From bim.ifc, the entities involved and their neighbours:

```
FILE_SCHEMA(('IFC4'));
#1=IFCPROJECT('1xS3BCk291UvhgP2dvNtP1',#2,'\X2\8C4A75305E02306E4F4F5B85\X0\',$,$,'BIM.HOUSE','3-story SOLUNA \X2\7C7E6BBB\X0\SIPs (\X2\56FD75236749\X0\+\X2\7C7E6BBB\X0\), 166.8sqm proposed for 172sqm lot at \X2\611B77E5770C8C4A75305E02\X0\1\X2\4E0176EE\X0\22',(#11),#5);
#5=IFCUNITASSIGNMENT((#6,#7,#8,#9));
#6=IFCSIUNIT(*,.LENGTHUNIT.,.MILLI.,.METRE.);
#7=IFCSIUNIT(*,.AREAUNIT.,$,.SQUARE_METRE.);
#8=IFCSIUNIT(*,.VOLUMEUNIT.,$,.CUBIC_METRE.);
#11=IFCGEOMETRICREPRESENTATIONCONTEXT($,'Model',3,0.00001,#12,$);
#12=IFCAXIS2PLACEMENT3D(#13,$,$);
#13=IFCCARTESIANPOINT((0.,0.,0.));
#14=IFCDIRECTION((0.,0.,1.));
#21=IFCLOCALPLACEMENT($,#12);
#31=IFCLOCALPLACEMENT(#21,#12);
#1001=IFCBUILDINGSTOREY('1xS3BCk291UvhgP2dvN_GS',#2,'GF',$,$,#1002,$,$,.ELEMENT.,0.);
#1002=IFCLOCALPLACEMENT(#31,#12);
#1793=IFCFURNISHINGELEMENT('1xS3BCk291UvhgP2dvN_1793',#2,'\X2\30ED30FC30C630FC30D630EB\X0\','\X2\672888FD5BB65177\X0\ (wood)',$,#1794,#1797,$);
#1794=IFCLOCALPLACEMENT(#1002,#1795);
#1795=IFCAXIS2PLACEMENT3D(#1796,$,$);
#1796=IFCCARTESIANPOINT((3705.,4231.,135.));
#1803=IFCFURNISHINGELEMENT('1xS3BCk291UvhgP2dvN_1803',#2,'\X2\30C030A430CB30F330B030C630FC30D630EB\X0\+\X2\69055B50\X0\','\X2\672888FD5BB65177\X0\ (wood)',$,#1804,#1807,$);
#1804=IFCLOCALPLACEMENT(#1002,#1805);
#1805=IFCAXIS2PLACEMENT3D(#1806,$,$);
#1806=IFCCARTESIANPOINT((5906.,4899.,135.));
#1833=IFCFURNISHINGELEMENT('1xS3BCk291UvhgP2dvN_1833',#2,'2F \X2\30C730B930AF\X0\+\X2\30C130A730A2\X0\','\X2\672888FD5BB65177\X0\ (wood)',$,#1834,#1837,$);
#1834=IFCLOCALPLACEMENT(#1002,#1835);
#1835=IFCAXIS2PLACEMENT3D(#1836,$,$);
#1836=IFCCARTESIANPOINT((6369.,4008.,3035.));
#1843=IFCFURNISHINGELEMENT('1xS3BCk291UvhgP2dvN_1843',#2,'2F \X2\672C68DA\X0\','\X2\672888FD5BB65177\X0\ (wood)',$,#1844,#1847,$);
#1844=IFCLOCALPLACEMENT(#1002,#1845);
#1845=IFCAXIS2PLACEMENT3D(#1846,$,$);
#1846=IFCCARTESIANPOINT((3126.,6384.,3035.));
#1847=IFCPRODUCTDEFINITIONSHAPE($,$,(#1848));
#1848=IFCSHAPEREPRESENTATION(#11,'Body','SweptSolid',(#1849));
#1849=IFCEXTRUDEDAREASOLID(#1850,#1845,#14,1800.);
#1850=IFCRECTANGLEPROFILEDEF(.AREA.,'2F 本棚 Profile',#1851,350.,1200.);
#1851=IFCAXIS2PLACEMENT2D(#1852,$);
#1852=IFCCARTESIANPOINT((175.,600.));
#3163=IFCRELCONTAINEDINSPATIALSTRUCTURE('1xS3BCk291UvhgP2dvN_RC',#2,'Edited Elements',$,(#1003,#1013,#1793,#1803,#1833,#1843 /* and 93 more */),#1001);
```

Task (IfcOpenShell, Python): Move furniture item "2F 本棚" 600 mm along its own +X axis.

```python
import ifcopenshell
import ifcopenshell.api.geometry
import ifcopenshell.util.placement

model = ifcopenshell.open("bim.ifc")

item = model.by_id(1843)
matrix = ifcopenshell.util.placement.get_local_placement(item.ObjectPlacement)
matrix[:3, 3] += matrix[:3, 0] * 600.0
ifcopenshell.api.geometry.edit_object_placement(model, product=item, matrix=matrix, is_si=False)

print(ifcopenshell.util.placement.get_local_placement(item.ObjectPlacement).round(3) + 0.0)

model.write("bim_v2.ifc")
```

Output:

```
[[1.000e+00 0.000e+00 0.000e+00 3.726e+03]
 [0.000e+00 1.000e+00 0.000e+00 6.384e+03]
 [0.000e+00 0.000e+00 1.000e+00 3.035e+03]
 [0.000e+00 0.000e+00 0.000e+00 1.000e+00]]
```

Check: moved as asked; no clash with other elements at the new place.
